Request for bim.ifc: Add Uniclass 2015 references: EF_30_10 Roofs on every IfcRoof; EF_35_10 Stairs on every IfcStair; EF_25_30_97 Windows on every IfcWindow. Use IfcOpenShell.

First a look at what the model holds.

```python
import ifcopenshell

model = ifcopenshell.open("bim.ifc")
print(model.schema)
print("classifications:", [c.Name for c in model.by_type("IfcClassification")])
for ifc_class in ("IfcDoor", "IfcRoof", "IfcStair", "IfcWall", "IfcWindow"):
    print(ifc_class, len(model.by_type(ifc_class)))
```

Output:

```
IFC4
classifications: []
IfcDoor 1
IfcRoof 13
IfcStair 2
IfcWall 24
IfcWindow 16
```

```python
import ifcopenshell
import ifcopenshell.api.classification

model = ifcopenshell.open("bim.ifc")

system = ifcopenshell.api.classification.add_classification(model, classification="Uniclass 2015")

codes = {
    "IfcRoof": ("EF_30_10", "Roofs"),
    "IfcStair": ("EF_35_10", "Stairs"),
    "IfcWindow": ("EF_25_30_97", "Windows"),
}
for ifc_class, (code, name) in codes.items():
    products = model.by_type(ifc_class)
    ifcopenshell.api.classification.add_reference(
        model, products=products, classification=system, identification=code, name=name
    )
    print(code, len(products))

model.write("bim_updated.ifc")
```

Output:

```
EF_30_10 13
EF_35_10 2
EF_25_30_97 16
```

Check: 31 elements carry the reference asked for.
